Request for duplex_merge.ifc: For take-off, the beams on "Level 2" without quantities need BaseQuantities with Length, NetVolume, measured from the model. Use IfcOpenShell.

First a look at what the model holds.

```python
import ifcopenshell
import ifcopenshell.util.element
import ifcopenshell.util.unit

model = ifcopenshell.open("duplex_merge.ifc")
print(model.schema)
for unit_type in ("LENGTHUNIT", "AREAUNIT", "VOLUMEUNIT"):
    print(unit_type, ifcopenshell.util.unit.calculate_unit_scale(model, unit_type))
storey = next(s for s in model.by_type("IfcBuildingStorey") if s.Name == "Level 2")
beams = [e for e in ifcopenshell.util.element.get_decomposition(storey) if e.is_a("IfcBeam")]
for e in sorted(beams, key=lambda e: e.id()):
    print(e.id(), e.is_a(), e.Name, list(ifcopenshell.util.element.get_psets(e, qtos_only=True)), sep=" | ")
```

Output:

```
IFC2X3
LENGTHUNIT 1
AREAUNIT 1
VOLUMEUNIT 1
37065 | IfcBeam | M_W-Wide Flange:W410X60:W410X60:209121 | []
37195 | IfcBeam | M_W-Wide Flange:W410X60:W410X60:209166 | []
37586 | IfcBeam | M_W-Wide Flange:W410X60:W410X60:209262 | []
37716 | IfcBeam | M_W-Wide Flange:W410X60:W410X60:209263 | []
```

```python
import ifcopenshell
import ifcopenshell.api.pset
import ifcopenshell.geom
import ifcopenshell.util.element
import ifcopenshell.util.shape
import ifcopenshell.util.unit

model = ifcopenshell.open("duplex_merge.ifc")
unit_scale = ifcopenshell.util.unit.calculate_unit_scale(model)
volume_scale = ifcopenshell.util.unit.calculate_unit_scale(model, "VOLUMEUNIT")
settings = ifcopenshell.geom.settings()

storey = next(s for s in model.by_type("IfcBuildingStorey") if s.Name == "Level 2")
beams = [e for e in ifcopenshell.util.element.get_decomposition(storey) if e.is_a("IfcBeam")]

for e in sorted(beams, key=lambda e: e.id()):
    if ifcopenshell.util.element.get_psets(e, qtos_only=True, should_inherit=False):
        continue
    # Geometry comes back in metres, in the element's own axes.
    shape = ifcopenshell.geom.create_shape(settings, e)
    values = {
        "Length": ifcopenshell.util.shape.get_max_xyz(shape.geometry) / unit_scale,
        "NetVolume": ifcopenshell.util.shape.get_volume(shape.geometry) / volume_scale,
    }
    qto = ifcopenshell.api.pset.add_qto(model, product=e, name="BaseQuantities")
    ifcopenshell.api.pset.edit_qto(model, qto=qto, properties=values)
    print(e.id(), {k: round(v, 3) for k, v in values.items()})

model.write("duplex_merge-out.ifc")
```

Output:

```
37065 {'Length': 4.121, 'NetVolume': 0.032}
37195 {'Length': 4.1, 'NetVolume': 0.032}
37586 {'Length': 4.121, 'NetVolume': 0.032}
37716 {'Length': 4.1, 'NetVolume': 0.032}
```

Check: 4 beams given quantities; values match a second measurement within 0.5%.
